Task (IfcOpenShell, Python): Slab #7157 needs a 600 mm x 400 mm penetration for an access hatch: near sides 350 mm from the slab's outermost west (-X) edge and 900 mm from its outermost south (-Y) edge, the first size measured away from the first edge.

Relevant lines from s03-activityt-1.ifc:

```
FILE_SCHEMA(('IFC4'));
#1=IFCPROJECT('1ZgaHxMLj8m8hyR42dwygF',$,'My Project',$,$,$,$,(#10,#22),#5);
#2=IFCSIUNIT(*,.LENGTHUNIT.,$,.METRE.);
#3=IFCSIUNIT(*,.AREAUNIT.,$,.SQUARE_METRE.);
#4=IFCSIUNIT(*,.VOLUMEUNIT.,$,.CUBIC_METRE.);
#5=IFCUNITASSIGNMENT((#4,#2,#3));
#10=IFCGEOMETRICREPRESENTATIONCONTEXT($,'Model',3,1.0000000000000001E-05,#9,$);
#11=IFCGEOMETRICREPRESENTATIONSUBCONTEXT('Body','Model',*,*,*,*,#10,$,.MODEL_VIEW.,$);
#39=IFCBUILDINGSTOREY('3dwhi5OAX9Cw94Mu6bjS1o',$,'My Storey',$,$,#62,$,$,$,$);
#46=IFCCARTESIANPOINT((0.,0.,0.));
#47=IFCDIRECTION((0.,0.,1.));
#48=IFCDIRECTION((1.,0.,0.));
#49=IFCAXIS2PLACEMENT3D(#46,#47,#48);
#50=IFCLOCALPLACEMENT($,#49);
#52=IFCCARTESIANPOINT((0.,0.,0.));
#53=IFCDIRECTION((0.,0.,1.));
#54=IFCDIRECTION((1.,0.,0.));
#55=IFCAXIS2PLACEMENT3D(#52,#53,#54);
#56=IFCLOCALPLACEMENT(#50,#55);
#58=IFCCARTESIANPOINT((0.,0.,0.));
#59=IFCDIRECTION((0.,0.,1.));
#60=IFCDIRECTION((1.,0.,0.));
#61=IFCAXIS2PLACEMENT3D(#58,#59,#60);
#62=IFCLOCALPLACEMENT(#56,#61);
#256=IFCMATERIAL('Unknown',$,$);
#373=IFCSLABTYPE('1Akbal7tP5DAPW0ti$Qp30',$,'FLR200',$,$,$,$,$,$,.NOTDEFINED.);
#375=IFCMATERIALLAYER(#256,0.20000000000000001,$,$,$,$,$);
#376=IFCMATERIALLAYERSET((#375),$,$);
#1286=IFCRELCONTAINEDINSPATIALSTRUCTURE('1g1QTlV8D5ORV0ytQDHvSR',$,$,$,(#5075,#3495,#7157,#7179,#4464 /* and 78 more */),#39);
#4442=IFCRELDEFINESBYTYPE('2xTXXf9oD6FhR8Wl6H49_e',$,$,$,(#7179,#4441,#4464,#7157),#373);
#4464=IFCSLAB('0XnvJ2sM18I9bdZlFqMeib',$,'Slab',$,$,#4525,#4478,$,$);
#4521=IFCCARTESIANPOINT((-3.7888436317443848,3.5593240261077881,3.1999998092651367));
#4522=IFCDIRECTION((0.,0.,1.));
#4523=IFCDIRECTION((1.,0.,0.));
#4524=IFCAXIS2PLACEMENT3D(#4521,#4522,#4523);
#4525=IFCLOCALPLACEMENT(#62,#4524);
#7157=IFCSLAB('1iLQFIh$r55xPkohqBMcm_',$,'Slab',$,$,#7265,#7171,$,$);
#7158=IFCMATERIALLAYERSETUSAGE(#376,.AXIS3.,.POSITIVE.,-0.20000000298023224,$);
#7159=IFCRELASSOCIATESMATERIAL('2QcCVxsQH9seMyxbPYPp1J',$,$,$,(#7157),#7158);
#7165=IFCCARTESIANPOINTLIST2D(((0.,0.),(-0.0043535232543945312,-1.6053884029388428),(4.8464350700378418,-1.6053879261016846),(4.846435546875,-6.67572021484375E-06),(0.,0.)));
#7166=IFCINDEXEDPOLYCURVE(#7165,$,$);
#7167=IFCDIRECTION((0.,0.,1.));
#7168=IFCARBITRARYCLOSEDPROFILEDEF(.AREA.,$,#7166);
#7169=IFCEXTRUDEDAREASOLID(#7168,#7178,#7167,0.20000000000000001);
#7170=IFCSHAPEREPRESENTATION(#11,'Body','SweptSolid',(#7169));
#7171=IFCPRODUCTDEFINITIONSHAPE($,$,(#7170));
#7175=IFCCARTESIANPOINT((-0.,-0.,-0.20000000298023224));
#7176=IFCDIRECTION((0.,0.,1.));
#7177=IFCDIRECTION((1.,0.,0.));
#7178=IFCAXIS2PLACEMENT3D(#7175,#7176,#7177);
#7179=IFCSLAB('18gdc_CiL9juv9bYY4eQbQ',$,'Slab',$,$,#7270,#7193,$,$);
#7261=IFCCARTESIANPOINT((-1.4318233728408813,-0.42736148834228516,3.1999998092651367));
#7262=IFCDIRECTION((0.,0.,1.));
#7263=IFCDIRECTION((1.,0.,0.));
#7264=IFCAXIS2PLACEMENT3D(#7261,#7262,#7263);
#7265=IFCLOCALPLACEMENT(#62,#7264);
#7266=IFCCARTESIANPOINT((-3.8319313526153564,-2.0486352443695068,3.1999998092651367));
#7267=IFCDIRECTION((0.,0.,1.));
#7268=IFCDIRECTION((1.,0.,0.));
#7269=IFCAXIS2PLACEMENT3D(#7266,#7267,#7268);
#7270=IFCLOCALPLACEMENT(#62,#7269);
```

```python
import numpy as np
import ifcopenshell
import ifcopenshell.api.feature
import ifcopenshell.api.geometry
import ifcopenshell.api.root
import ifcopenshell.geom
import ifcopenshell.util.placement
import ifcopenshell.util.representation
import ifcopenshell.util.shape
import ifcopenshell.util.unit

model = ifcopenshell.open("s03-activityt-1.ifc")
unit_scale = ifcopenshell.util.unit.calculate_unit_scale(model)
settings = ifcopenshell.geom.settings()


def volume(element):
    """Net volume in cubic metres, openings subtracted."""
    shape = ifcopenshell.geom.create_shape(settings, element)
    return ifcopenshell.util.shape.get_volume(shape.geometry)


slab = model.by_guid("1iLQFIh$r55xPkohqBMcm_")
before = volume(slab)

# Extent in the slab's own axes, in metres. The edges named are its -X and -Y sides.
slab_shape = ifcopenshell.geom.create_shape(settings, slab)
vertices = ifcopenshell.util.shape.get_vertices(slab_shape.geometry)
x_min, y_min, bottom = vertices.min(axis=0)
top = vertices[:, 2].max()

opening = ifcopenshell.api.root.create_entity(model, ifc_class="IfcOpeningElement", name="Access hatch opening", predefined_type="OPENING")
context = ifcopenshell.util.representation.get_context(model, "Model", "Body", "MODEL_VIEW")
width, depth = 0.6, 0.4
outline = [(0.0, 0.0), (width, 0.0), (width, depth), (0.0, depth), (0.0, 0.0)]
# Overshoot both faces by 50 mm so the cut is clean.
shape = ifcopenshell.api.geometry.add_slab_representation(
    model, context=context, depth=top - bottom + 0.1, polyline=outline
)
ifcopenshell.api.geometry.assign_representation(model, product=opening, representation=shape)

matrix = ifcopenshell.util.placement.get_local_placement(slab.ObjectPlacement)
matrix[:, 3] = matrix @ np.append(np.array([x_min + 0.35, y_min + 0.9, bottom - 0.05]) / unit_scale, 1.0)
ifcopenshell.api.geometry.edit_object_placement(model, product=opening, matrix=matrix, is_si=False)
ifcopenshell.api.feature.add_feature(model, feature=opening, element=slab)

after = volume(slab)

print(f"slab volume {before:.3f} -> {after:.3f} m3")

model.write("s03-activityt-1_rev.ifc")
```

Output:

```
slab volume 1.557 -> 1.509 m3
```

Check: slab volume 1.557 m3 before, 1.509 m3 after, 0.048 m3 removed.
